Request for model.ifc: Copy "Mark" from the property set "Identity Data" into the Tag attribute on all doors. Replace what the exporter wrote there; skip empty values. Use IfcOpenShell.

First a look at what the model holds.

```python
import ifcopenshell
import ifcopenshell.util.element

model = ifcopenshell.open("model.ifc")
print(model.schema)
doors = model.by_type("IfcDoor")
print(len(doors), "doors")
for e in doors[:8]:
    source = ifcopenshell.util.element.get_pset(e, "Identity Data", "Mark")
    target = e.Tag
    print(e.id(), repr(source), repr(target), sep=" | ")
```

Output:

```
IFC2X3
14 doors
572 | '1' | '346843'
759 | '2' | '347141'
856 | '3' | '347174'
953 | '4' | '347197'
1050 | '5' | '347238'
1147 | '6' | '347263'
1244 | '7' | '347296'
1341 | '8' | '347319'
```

```python
import ifcopenshell
import ifcopenshell.util.element

model = ifcopenshell.open("model.ifc")

count = 0
for e in model.by_type("IfcDoor"):
    value = ifcopenshell.util.element.get_pset(e, "Identity Data", "Mark")
    current = e.Tag
    if not value or not value.strip() or current == value:
        continue
    e.Tag = value
    count += 1

print(count, "doors updated")

model.write("model_updated.ifc")
```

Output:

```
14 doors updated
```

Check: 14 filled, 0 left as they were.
